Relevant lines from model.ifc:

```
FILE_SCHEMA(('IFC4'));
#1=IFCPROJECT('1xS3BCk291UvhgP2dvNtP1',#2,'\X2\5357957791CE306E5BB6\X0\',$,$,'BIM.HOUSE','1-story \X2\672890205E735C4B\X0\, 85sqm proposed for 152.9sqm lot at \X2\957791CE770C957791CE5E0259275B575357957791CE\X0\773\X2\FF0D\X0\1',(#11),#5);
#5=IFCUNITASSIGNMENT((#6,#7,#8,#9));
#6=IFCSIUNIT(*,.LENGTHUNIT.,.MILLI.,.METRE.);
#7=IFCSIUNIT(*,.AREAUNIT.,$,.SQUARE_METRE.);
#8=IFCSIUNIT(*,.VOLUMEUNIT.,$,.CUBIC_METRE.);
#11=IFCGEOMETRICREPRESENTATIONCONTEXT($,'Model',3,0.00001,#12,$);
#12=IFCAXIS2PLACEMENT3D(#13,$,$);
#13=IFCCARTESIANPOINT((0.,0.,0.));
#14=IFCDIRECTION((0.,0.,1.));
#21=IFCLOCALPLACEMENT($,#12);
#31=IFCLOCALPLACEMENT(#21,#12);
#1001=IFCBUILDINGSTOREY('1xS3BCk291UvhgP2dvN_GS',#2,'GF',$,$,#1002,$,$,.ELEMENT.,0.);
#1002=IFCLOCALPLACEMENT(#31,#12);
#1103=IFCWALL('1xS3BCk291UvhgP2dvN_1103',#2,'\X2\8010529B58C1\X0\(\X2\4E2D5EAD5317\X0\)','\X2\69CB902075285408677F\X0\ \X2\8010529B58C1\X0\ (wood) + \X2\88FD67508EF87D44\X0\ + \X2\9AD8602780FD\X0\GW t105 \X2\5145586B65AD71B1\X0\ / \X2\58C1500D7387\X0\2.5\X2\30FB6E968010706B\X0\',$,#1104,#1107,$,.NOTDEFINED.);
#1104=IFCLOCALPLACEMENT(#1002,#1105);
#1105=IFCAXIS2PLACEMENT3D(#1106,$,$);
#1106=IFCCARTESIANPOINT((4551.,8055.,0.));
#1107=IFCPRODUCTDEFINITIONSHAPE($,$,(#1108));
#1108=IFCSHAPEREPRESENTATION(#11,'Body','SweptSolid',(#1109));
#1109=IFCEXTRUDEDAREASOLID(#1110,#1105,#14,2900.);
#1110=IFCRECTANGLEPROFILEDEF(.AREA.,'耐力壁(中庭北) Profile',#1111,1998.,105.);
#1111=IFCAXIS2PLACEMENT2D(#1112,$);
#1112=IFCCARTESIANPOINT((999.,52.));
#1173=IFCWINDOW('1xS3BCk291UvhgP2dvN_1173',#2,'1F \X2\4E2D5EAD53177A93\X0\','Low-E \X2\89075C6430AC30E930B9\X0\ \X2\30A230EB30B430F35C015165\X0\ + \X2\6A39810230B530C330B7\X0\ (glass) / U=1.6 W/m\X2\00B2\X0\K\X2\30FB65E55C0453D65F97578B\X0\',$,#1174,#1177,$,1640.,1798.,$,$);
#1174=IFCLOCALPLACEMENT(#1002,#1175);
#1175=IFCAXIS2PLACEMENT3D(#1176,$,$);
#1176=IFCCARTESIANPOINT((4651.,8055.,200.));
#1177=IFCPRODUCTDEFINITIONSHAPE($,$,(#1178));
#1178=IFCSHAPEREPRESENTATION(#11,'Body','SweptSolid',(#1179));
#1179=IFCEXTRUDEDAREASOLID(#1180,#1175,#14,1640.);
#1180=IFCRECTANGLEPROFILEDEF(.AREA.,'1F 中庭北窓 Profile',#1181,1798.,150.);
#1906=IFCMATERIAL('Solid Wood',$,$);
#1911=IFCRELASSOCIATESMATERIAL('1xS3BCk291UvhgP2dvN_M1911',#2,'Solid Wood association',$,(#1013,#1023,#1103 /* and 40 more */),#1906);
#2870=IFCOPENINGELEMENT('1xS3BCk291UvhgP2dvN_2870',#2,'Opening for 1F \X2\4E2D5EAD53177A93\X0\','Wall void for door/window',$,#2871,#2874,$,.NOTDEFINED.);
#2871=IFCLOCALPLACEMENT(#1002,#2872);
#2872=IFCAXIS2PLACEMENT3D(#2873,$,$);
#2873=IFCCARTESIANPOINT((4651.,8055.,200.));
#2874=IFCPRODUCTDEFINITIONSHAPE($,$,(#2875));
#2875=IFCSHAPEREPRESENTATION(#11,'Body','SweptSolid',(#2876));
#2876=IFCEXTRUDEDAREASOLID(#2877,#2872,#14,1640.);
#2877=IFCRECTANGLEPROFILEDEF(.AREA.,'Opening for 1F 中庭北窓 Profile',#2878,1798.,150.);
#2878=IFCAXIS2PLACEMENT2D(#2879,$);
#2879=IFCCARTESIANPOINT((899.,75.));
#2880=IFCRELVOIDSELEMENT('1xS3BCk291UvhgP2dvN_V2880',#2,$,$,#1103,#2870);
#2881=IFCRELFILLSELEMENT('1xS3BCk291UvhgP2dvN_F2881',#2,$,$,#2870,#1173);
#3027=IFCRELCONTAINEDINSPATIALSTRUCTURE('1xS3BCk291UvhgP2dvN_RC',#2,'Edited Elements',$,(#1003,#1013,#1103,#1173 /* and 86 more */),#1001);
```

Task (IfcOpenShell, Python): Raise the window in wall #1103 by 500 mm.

```python
import numpy as np
import ifcopenshell
import ifcopenshell.api.geometry
import ifcopenshell.util.placement
import ifcopenshell.util.unit

model = ifcopenshell.open("model.ifc")
unit_scale = ifcopenshell.util.unit.calculate_unit_scale(model)

window = model.by_id(1173)
opening = window.FillsVoids[0].RelatingOpeningElement
dz = 0.5 / unit_scale

shift = np.array([0.0, 0.0, dz])
# The window is not placed relative to its opening, so move both.
for product in (opening, window):
    matrix = ifcopenshell.util.placement.get_local_placement(product.ObjectPlacement)
    matrix[:3, 3] += shift
    ifcopenshell.api.geometry.edit_object_placement(model, product=product, matrix=matrix, is_si=False)

print(f"moved by {dz * unit_scale:+.3f} m")

model.write("model-out.ifc")
```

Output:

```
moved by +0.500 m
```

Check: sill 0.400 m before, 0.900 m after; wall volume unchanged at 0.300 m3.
